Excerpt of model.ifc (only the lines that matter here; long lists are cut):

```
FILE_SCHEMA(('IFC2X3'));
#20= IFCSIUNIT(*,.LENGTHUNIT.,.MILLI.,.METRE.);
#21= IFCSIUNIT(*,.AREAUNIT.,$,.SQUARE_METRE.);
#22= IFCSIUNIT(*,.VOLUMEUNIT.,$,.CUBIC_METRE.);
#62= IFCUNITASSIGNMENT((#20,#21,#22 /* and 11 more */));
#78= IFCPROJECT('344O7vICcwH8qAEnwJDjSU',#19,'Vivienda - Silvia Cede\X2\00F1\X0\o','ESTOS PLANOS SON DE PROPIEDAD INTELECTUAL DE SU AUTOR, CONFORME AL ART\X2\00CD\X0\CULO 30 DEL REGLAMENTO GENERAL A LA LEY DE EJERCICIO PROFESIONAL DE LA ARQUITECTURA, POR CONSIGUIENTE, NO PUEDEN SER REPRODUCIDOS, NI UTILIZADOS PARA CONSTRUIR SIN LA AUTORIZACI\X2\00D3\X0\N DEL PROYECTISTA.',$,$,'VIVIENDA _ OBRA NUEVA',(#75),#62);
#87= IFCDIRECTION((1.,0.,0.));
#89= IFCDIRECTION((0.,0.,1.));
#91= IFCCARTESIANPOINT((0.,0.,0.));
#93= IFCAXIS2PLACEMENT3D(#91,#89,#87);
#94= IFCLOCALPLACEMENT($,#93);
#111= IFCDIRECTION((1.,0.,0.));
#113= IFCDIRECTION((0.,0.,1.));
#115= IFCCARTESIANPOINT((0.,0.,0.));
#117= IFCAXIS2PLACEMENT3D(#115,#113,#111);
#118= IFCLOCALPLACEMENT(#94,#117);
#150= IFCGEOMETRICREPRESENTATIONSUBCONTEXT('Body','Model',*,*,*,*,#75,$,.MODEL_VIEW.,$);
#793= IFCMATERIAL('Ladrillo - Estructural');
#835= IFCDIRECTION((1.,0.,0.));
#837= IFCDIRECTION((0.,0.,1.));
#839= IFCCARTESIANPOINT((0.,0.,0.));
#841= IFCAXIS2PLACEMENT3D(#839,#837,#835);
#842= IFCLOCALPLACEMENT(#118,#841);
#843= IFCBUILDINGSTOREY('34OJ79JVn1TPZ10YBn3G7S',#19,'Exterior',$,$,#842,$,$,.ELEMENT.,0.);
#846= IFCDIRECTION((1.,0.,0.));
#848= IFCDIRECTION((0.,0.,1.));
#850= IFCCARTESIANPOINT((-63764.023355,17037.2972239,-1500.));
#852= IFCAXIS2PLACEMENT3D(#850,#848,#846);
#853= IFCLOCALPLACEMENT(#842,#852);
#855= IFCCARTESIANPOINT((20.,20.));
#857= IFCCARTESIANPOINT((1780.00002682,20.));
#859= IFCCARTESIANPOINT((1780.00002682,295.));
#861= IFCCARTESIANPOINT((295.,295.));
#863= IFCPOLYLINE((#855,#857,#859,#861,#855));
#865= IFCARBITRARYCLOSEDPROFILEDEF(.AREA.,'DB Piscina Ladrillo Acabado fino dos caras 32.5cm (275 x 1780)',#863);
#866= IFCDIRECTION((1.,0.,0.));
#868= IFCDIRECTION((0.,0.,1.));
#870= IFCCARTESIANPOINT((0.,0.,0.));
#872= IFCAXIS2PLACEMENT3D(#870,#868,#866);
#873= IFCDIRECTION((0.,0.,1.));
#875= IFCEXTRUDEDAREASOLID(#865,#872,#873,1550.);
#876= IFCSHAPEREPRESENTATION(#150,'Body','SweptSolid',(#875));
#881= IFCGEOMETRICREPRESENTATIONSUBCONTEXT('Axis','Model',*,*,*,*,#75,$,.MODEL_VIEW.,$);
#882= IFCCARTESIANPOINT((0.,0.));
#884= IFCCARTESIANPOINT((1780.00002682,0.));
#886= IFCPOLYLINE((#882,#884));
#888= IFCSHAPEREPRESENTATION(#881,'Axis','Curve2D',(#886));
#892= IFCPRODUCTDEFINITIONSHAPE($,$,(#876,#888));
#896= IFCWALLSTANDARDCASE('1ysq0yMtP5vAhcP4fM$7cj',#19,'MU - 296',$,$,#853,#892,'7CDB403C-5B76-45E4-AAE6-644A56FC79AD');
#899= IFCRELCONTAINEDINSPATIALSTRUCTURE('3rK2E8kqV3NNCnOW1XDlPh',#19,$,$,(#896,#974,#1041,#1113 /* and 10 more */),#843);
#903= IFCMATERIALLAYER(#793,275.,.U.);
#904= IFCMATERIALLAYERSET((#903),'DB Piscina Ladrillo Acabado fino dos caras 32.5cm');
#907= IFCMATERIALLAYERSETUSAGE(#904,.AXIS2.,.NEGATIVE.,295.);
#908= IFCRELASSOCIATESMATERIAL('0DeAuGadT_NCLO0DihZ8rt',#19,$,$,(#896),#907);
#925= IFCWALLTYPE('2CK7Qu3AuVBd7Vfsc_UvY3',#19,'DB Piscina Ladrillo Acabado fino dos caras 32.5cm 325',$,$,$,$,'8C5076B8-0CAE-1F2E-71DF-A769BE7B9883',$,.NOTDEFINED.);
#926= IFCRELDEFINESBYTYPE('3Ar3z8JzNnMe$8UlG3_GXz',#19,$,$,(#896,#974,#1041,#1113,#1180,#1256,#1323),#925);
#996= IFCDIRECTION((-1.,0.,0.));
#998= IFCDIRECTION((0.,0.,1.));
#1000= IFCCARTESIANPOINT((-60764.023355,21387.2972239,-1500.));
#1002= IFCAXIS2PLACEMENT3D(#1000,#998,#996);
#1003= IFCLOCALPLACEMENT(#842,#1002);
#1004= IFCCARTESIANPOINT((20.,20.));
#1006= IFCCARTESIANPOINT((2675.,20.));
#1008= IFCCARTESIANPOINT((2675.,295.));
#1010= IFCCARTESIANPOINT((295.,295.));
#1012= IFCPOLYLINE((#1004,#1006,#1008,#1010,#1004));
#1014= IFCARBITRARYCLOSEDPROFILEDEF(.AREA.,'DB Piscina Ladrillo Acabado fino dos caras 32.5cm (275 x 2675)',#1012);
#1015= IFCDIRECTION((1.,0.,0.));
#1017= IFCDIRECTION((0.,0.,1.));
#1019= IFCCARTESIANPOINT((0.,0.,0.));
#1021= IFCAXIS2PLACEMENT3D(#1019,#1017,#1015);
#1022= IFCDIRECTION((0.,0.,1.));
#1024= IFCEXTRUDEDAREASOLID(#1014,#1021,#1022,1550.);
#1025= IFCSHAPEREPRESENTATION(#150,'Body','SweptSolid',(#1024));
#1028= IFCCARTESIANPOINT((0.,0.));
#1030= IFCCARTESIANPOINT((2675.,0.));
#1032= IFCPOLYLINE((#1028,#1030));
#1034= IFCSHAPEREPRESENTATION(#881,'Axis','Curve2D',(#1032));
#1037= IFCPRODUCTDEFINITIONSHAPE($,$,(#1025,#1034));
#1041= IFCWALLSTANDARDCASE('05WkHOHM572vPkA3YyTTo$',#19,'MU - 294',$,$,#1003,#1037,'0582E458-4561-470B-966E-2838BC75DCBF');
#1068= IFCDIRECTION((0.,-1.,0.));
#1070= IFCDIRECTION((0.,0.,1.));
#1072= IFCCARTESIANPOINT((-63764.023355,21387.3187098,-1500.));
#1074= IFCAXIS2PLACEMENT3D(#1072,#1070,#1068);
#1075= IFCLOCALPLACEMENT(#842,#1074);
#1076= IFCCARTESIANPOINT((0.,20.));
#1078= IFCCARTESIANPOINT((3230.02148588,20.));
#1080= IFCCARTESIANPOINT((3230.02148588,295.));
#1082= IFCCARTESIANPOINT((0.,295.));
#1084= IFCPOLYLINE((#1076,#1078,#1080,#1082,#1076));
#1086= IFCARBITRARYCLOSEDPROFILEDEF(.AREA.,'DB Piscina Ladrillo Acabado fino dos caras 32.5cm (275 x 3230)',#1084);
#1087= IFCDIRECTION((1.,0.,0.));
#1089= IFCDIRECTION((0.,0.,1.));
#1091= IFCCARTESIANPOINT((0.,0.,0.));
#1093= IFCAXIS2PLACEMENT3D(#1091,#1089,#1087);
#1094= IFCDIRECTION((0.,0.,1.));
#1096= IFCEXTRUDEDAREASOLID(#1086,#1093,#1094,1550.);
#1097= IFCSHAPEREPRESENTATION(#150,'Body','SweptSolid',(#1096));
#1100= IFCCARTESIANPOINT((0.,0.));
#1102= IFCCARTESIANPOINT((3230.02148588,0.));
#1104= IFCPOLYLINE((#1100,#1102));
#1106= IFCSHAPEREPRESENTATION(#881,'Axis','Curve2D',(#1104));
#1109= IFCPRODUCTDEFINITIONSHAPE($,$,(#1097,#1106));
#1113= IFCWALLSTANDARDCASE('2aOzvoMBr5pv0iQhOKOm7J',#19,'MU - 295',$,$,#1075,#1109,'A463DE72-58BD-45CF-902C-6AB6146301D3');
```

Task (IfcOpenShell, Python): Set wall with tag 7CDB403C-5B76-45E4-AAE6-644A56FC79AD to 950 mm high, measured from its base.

```python
import ifcopenshell
import ifcopenshell.geom
import ifcopenshell.util.representation
import ifcopenshell.util.shape

model = ifcopenshell.open("model.ifc")
settings = ifcopenshell.geom.settings()


def volume(element):
    """Net volume in cubic metres, openings subtracted."""
    shape = ifcopenshell.geom.create_shape(settings, element)
    return ifcopenshell.util.shape.get_volume(shape.geometry)


wall = model.by_guid("1ysq0yMtP5vAhcP4fM$7cj")
before = volume(wall)

body = ifcopenshell.util.representation.get_representation(wall, "Model", "Body")
solid = body.Items[0]
old_height = solid.Depth
solid.Depth = 950.0
after = volume(wall)

print(f"height {old_height:g} -> {solid.Depth:g}, volume {before:.3f} -> {after:.3f} m3")

model.write("model_edited.ifc")
```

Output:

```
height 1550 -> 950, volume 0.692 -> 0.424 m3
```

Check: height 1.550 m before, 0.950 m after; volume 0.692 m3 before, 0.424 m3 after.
